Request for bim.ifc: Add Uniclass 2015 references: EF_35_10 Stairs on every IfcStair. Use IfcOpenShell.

First a look at what the model holds.

```python
import ifcopenshell

model = ifcopenshell.open("bim.ifc")
print(model.schema)
print("classifications:", [c.Name for c in model.by_type("IfcClassification")])
for ifc_class in ("IfcDoor", "IfcRoof", "IfcStair", "IfcWall", "IfcWindow"):
    print(ifc_class, len(model.by_type(ifc_class)))
```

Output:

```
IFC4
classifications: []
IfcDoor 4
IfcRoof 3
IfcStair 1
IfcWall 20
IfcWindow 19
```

```python
import ifcopenshell
import ifcopenshell.api.classification

model = ifcopenshell.open("bim.ifc")

system = ifcopenshell.api.classification.add_classification(model, classification="Uniclass 2015")

codes = {
    "IfcStair": ("EF_35_10", "Stairs"),
}
for ifc_class, (code, name) in codes.items():
    products = model.by_type(ifc_class)
    ifcopenshell.api.classification.add_reference(
        model, products=products, classification=system, identification=code, name=name
    )
    print(code, len(products))

model.write("bim_rev.ifc")
```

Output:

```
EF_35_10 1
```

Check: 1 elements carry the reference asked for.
